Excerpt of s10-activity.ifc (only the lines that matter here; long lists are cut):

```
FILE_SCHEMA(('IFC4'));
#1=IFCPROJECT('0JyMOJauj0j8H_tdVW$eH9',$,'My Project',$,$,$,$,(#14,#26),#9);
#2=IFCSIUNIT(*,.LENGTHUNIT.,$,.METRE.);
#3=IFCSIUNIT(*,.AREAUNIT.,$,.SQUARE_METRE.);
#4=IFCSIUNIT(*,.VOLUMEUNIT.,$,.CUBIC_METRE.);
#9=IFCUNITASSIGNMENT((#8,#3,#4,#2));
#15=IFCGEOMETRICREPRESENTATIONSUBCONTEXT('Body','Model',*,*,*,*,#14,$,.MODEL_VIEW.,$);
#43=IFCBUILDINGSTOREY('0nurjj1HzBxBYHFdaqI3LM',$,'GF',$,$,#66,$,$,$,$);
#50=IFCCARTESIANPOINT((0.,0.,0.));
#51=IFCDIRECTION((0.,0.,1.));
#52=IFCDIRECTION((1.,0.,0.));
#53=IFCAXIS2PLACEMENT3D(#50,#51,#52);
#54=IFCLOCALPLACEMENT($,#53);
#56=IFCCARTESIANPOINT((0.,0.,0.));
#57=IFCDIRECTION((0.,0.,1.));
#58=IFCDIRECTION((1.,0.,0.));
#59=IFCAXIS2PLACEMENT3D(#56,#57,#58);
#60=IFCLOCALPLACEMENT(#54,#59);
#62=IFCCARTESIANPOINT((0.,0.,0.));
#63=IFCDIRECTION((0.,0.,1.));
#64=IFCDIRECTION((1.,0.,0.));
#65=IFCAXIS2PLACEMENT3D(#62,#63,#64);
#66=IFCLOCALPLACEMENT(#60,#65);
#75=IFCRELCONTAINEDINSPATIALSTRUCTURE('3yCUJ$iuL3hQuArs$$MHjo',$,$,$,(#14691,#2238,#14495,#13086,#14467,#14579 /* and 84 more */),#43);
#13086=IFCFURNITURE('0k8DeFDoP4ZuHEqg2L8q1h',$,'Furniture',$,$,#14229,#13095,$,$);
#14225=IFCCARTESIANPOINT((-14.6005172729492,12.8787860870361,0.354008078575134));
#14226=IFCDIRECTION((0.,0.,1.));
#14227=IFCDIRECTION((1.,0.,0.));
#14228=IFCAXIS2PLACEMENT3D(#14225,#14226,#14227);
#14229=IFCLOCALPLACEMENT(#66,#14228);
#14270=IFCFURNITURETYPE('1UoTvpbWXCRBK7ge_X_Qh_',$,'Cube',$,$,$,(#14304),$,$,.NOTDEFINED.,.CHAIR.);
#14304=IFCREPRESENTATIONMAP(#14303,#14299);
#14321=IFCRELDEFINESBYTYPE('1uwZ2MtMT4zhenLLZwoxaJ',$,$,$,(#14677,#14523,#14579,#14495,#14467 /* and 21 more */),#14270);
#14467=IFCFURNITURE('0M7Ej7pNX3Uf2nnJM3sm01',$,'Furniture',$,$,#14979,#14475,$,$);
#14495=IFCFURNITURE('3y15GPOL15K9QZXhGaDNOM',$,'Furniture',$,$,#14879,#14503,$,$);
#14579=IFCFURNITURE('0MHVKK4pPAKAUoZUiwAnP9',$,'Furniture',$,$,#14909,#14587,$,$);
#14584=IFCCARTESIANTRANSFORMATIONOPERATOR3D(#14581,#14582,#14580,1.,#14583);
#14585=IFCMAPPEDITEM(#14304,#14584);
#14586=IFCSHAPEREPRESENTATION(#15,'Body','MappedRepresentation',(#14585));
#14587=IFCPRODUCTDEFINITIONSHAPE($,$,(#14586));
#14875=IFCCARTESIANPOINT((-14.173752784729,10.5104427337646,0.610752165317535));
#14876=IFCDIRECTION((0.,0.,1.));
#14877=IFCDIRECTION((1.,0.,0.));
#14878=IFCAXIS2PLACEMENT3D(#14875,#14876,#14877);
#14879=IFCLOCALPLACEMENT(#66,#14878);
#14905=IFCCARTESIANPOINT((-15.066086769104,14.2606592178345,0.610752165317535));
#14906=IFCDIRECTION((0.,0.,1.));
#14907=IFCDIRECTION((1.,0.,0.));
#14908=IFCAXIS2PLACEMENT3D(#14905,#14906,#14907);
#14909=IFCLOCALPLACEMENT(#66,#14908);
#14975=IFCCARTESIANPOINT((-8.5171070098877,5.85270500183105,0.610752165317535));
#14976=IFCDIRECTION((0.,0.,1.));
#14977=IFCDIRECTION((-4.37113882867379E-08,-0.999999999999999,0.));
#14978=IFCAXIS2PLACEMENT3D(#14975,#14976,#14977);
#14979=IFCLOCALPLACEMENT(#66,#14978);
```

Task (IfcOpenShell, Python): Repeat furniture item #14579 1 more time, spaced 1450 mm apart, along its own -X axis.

```python
import ifcopenshell
import ifcopenshell.api.geometry
import ifcopenshell.api.root
import ifcopenshell.util.element
import ifcopenshell.util.placement
import ifcopenshell.util.unit

model = ifcopenshell.open("s10-activity.ifc")
unit_scale = ifcopenshell.util.unit.calculate_unit_scale(model)

source = model.by_guid("0MHVKK4pPAKAUoZUiwAnP9")
base = ifcopenshell.util.placement.get_local_placement(source.ObjectPlacement)
step = -base[:3, 0] * 1.45 / unit_scale

for i in range(1, 2):
    copy = ifcopenshell.api.root.copy_class(model, product=source)
    copy.Representation = ifcopenshell.util.element.copy_deep(
        model, source.Representation, exclude=["IfcGeometricRepresentationContext", "IfcRepresentationMap"]
    )
    matrix = base.copy()
    matrix[:3, 3] += i * step
    print("added at", matrix[:3, 3].round(3) + 0.0)
    ifcopenshell.api.geometry.edit_object_placement(model, product=copy, matrix=matrix, is_si=False)

model.write("s10-activity_rev.ifc")
```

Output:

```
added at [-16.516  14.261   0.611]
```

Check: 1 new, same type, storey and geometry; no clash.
